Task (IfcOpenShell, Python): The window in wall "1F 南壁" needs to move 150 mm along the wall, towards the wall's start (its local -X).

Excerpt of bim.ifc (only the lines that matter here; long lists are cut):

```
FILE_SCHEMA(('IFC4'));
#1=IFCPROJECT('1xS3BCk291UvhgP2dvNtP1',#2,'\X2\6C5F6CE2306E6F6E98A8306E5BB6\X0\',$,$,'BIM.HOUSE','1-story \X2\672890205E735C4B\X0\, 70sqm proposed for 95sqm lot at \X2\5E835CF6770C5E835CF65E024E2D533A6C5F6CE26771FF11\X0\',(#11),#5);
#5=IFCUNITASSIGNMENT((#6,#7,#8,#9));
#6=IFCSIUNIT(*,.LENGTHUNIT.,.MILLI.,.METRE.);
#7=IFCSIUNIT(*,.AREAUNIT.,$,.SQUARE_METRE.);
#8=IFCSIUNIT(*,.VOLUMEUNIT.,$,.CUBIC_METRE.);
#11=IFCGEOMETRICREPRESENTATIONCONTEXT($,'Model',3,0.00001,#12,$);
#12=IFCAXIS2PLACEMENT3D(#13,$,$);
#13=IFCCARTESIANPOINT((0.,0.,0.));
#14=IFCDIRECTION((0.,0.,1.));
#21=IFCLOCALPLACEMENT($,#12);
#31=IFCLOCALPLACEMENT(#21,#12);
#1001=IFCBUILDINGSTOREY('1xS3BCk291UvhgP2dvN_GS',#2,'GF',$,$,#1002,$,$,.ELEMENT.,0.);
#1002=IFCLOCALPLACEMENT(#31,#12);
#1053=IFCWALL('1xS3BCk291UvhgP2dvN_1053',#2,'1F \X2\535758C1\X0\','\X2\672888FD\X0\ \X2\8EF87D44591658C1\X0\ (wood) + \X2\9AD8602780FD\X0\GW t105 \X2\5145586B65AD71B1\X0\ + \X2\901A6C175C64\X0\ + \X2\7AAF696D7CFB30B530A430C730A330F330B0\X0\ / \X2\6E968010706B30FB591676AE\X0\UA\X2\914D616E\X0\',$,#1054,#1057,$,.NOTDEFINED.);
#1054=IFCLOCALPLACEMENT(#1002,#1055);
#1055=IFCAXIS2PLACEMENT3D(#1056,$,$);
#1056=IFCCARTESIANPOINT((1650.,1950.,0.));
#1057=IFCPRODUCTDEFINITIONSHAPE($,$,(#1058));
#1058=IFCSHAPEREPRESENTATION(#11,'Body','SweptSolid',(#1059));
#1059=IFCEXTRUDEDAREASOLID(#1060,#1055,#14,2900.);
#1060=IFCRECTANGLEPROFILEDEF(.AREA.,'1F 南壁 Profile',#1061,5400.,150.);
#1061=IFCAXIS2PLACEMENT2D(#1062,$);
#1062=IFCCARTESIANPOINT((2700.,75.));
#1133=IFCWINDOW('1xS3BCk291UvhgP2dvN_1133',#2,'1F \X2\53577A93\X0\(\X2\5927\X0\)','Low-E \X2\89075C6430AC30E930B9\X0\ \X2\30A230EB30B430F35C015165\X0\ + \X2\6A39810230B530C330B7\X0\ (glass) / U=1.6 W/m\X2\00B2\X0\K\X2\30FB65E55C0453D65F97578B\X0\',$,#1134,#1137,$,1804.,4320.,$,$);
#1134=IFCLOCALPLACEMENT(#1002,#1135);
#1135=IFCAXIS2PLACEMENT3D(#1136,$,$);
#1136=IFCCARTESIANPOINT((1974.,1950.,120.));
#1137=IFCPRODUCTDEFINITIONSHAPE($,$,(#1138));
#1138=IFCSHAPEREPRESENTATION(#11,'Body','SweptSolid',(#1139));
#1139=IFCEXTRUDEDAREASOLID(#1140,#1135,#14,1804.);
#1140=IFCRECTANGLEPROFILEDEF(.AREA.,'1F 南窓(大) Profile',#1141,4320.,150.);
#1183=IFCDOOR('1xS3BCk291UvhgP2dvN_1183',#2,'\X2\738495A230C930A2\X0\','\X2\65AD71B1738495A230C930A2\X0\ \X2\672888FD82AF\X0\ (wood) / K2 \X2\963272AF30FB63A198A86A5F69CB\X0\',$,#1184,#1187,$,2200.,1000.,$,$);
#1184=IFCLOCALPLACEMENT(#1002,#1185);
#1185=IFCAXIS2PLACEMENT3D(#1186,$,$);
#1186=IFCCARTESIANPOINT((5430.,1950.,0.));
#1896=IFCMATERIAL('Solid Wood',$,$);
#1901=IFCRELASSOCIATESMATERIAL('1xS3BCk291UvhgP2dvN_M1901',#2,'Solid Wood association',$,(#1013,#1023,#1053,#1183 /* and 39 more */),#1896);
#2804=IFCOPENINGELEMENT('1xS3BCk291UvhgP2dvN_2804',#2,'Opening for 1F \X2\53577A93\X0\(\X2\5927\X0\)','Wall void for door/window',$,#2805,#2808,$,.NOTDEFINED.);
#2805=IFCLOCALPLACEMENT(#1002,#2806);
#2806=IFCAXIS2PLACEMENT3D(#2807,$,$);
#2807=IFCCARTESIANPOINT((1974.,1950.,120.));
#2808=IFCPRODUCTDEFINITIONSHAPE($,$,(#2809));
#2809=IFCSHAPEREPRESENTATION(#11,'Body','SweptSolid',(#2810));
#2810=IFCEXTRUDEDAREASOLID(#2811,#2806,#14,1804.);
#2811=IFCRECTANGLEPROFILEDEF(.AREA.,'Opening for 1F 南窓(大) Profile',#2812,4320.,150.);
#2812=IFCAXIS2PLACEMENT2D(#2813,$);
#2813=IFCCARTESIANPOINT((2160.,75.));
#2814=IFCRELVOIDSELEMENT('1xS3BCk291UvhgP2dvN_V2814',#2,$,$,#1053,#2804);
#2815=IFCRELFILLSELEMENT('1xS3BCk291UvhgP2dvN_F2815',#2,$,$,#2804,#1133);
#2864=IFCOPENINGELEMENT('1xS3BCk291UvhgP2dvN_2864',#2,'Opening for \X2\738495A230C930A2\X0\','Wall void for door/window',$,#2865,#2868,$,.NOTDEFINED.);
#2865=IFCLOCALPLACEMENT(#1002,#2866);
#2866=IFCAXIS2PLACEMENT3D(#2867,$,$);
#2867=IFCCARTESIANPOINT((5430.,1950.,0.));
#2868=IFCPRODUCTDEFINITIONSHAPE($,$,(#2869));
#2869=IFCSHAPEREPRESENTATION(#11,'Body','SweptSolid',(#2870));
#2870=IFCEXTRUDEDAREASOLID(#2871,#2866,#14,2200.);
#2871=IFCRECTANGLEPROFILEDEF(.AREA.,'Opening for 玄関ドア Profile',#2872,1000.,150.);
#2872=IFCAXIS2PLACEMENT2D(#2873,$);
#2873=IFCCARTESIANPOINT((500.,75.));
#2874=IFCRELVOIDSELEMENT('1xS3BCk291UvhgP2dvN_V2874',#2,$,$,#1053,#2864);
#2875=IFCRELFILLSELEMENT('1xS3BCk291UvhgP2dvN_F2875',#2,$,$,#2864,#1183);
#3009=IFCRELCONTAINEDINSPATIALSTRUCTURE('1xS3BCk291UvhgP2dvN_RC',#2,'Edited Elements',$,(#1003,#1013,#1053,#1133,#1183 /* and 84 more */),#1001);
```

```python
import ifcopenshell
import ifcopenshell.api.geometry
import ifcopenshell.util.placement

model = ifcopenshell.open("bim.ifc")

window = model.by_guid("1xS3BCk291UvhgP2dvN_1133")
opening = window.FillsVoids[0].RelatingOpeningElement
wall = opening.VoidsElements[0].RelatingBuildingElement

wall_matrix = ifcopenshell.util.placement.get_local_placement(wall.ObjectPlacement)
shift = wall_matrix[:3, 0] * -150.0
before = ifcopenshell.util.placement.get_local_placement(window.ObjectPlacement)[:3, 3].copy()

# The window is not placed relative to its opening, so move both.
for product in (opening, window):
    matrix = ifcopenshell.util.placement.get_local_placement(product.ObjectPlacement)
    matrix[:3, 3] += shift
    ifcopenshell.api.geometry.edit_object_placement(model, product=product, matrix=matrix, is_si=False)

after = ifcopenshell.util.placement.get_local_placement(window.ObjectPlacement)[:3, 3]
print("window moved by", (after - before).round(3) + 0.0)

model.write("bim-out.ifc")
```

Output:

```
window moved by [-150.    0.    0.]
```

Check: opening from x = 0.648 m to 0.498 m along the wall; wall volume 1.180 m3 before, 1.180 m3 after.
